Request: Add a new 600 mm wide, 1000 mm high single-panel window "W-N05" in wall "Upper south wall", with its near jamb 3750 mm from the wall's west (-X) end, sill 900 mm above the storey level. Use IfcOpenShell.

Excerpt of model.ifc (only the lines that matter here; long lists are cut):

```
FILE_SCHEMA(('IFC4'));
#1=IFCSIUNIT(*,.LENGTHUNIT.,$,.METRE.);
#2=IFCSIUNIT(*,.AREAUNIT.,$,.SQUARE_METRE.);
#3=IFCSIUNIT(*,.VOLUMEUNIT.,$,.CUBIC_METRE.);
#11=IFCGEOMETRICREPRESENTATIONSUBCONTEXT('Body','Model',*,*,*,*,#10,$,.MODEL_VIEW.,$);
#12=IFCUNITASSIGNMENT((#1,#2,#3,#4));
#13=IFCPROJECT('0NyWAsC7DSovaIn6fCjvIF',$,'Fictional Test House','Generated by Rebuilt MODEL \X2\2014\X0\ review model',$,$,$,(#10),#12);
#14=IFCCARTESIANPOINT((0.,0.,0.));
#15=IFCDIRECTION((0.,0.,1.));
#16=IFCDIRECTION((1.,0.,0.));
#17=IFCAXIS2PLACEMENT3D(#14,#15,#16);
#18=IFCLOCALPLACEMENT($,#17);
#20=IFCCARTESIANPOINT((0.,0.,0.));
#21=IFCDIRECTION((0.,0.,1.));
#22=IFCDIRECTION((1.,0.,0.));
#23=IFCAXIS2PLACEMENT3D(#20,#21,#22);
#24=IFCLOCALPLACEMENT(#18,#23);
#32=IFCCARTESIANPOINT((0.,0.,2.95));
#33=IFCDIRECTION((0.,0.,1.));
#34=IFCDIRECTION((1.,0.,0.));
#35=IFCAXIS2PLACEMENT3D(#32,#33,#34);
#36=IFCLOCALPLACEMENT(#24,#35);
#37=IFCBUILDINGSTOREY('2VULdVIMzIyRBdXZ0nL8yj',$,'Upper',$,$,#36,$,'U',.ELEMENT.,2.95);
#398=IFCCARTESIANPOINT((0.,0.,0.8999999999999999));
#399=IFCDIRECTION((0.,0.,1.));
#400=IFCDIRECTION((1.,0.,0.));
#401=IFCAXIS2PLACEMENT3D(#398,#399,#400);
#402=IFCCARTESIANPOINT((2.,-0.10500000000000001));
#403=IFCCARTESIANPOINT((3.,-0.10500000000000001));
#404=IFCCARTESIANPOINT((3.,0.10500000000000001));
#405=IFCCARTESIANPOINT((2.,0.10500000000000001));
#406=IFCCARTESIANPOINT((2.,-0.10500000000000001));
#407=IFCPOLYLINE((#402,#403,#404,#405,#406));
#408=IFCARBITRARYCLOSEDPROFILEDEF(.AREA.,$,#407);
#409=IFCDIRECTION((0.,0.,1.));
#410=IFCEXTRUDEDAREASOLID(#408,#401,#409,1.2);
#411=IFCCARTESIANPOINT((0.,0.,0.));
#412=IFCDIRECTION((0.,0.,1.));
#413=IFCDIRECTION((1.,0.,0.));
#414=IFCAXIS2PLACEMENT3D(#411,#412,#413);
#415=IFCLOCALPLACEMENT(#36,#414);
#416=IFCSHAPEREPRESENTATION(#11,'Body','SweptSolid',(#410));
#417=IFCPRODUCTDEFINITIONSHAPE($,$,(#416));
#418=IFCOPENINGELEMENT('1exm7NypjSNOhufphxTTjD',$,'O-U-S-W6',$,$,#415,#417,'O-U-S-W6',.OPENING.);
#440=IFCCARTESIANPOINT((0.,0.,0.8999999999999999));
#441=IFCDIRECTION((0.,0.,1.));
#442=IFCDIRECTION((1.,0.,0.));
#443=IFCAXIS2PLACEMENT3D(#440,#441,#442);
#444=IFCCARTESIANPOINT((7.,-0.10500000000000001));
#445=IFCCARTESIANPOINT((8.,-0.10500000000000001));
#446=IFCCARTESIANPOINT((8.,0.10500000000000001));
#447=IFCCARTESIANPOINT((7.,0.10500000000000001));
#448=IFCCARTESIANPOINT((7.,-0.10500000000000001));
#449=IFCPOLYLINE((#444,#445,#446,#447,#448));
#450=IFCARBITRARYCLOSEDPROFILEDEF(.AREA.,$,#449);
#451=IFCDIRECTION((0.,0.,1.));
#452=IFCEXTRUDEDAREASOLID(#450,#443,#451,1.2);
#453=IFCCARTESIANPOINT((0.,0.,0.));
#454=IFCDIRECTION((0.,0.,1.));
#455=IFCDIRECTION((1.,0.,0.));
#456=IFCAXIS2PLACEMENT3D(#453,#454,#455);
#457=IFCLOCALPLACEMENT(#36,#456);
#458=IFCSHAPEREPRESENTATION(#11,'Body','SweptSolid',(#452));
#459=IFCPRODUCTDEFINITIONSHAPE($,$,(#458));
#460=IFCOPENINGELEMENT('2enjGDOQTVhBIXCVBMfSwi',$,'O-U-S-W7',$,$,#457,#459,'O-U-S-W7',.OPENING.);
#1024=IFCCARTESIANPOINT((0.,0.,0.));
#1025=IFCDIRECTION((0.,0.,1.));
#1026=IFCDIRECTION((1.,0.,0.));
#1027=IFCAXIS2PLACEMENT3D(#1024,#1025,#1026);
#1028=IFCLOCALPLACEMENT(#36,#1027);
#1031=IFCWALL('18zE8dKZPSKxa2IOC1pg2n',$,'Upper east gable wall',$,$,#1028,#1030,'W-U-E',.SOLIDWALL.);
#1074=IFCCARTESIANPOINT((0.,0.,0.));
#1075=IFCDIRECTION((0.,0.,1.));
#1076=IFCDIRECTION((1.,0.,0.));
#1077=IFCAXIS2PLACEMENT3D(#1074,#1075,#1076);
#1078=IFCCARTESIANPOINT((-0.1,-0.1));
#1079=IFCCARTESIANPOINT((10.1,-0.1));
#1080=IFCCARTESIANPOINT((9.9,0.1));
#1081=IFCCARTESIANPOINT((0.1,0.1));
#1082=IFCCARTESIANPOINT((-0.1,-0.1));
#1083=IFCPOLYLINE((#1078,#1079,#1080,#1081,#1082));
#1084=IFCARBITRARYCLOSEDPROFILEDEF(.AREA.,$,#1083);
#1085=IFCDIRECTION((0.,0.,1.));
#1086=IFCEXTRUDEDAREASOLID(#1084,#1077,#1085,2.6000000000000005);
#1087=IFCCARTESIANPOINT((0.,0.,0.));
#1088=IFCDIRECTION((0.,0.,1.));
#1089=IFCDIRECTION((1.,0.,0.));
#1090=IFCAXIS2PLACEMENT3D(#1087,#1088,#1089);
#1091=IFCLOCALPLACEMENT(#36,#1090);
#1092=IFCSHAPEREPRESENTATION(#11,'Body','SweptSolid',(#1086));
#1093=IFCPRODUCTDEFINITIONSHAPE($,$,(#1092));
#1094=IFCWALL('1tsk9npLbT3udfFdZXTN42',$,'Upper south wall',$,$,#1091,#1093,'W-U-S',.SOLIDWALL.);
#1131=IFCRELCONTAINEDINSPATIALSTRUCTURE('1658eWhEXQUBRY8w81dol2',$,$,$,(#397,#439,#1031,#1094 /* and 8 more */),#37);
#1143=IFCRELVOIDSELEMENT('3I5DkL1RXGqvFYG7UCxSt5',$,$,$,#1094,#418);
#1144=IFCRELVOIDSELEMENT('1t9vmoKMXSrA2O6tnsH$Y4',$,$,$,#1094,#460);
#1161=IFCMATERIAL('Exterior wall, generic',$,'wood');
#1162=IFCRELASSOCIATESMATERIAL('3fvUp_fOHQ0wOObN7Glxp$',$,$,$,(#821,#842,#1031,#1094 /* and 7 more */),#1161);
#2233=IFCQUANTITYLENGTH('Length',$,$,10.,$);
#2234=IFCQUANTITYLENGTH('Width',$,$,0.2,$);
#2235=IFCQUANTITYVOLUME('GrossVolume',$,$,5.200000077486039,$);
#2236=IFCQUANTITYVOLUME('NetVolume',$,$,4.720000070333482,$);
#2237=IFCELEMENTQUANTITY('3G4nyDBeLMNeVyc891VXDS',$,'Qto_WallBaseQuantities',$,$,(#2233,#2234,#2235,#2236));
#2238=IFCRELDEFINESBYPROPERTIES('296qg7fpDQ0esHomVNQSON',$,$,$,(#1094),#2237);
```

```python
import numpy as np
import ifcopenshell
import ifcopenshell.api.feature
import ifcopenshell.api.geometry
import ifcopenshell.api.pset
import ifcopenshell.api.root
import ifcopenshell.api.spatial
import ifcopenshell.geom
import ifcopenshell.util.element
import ifcopenshell.util.placement
import ifcopenshell.util.representation
import ifcopenshell.util.shape
import ifcopenshell.util.unit

model = ifcopenshell.open("model.ifc")
unit_scale = ifcopenshell.util.unit.calculate_unit_scale(model)
volume_scale = ifcopenshell.util.unit.calculate_unit_scale(model, "VOLUMEUNIT")
settings = ifcopenshell.geom.settings()


def volume(element):
    """Net volume in cubic metres, openings subtracted."""
    shape = ifcopenshell.geom.create_shape(settings, element)
    return ifcopenshell.util.shape.get_volume(shape.geometry)


wall = model.by_id(1094)
storey = ifcopenshell.util.element.get_container(wall, ifc_class="IfcBuildingStorey")
context = ifcopenshell.util.representation.get_context(model, "Model", "Body", "MODEL_VIEW")
before = volume(wall)

width, height, from_end, sill = 0.6, 1, 3.75, 0.9  # metres

# The wall runs along its own X axis, and the end named is its -X end.
wall_shape = ifcopenshell.geom.create_shape(settings, wall)
x, y, z = ifcopenshell.util.shape.get_vertices(wall_shape.geometry).T
start = x.min() + from_end
face, thickness = float(y.min()), float(y.max() - y.min())
wall_matrix = ifcopenshell.util.placement.get_local_placement(wall.ObjectPlacement)
level = ifcopenshell.util.placement.get_local_placement(storey.ObjectPlacement)[2, 3]


def in_wall(x, y):
    """Placement at x, y metres in the wall's axes, at sill height."""
    matrix = wall_matrix.copy()
    matrix[:, 3] = wall_matrix @ np.array([x / unit_scale, y / unit_scale, 0.0, 1.0])
    matrix[2, 3] = level + sill / unit_scale
    return matrix


# Opening: a box that overshoots both wall faces by 50 mm.
opening = ifcopenshell.api.root.create_entity(model, ifc_class="IfcOpeningElement", predefined_type="OPENING")
box = ifcopenshell.api.geometry.add_wall_representation(
    model, context=context, length=width, height=height, thickness=thickness + 0.1
)
ifcopenshell.api.geometry.assign_representation(model, product=opening, representation=box)
ifcopenshell.api.geometry.edit_object_placement(model, product=opening, matrix=in_wall(start, face - 0.05), is_si=False)
ifcopenshell.api.feature.add_feature(model, feature=opening, element=wall)

window = ifcopenshell.api.root.create_entity(model, ifc_class="IfcWindow", name="W-N05", predefined_type="WINDOW")
window.OverallWidth, window.OverallHeight = width / unit_scale, height / unit_scale
window.PartitioningType = "SINGLE_PANEL"
body = ifcopenshell.api.geometry.add_window_representation(
    model,
    context=context,
    overall_width=window.OverallWidth,
    overall_height=window.OverallHeight,
    partition_type="SINGLE_PANEL",
)
ifcopenshell.api.geometry.assign_representation(model, product=window, representation=body)
ifcopenshell.api.spatial.assign_container(model, products=[window], relating_structure=storey)
ifcopenshell.api.feature.add_filling(model, opening=opening, element=window)

# Centre the window in the wall's thickness.
ifcopenshell.api.geometry.edit_object_placement(model, product=window, matrix=in_wall(start, face), is_si=False)
window_shape = ifcopenshell.geom.create_shape(settings, window)
depth = ifcopenshell.util.shape.get_vertices(window_shape.geometry)[:, 1]
offset = face + thickness / 2 - (depth.min() + depth.max()) / 2
ifcopenshell.api.geometry.edit_object_placement(model, product=window, matrix=in_wall(start, offset), is_si=False)

after = volume(wall)

# Update the wall's stored quantities.
qto = model.by_id(ifcopenshell.util.element.get_pset(wall, "Qto_WallBaseQuantities", should_inherit=False)["id"])
ifcopenshell.api.pset.edit_qto(model, qto=qto, properties={"NetVolume": after / volume_scale})

print(f"wall volume {before:.3f} -> {after:.3f} m3")

model.write("model_edited.ifc")
```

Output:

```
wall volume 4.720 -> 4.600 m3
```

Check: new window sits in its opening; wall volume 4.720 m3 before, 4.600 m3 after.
